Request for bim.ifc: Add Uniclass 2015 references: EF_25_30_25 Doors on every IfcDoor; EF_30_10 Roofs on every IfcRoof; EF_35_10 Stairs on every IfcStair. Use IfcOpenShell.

First a look at what the model holds.

```python
import ifcopenshell

model = ifcopenshell.open("bim.ifc")
print(model.schema)
print("classifications:", [c.Name for c in model.by_type("IfcClassification")])
for ifc_class in ("IfcDoor", "IfcRoof", "IfcStair", "IfcWall", "IfcWindow"):
    print(ifc_class, len(model.by_type(ifc_class)))
```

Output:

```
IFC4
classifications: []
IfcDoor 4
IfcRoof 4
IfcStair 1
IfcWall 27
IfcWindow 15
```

```python
import ifcopenshell
import ifcopenshell.api.classification

model = ifcopenshell.open("bim.ifc")

system = ifcopenshell.api.classification.add_classification(model, classification="Uniclass 2015")

codes = {
    "IfcDoor": ("EF_25_30_25", "Doors"),
    "IfcRoof": ("EF_30_10", "Roofs"),
    "IfcStair": ("EF_35_10", "Stairs"),
}
for ifc_class, (code, name) in codes.items():
    products = model.by_type(ifc_class)
    ifcopenshell.api.classification.add_reference(
        model, products=products, classification=system, identification=code, name=name
    )
    print(code, len(products))

model.write("bim_updated.ifc")
```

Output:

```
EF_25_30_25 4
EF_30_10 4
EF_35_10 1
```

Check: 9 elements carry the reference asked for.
